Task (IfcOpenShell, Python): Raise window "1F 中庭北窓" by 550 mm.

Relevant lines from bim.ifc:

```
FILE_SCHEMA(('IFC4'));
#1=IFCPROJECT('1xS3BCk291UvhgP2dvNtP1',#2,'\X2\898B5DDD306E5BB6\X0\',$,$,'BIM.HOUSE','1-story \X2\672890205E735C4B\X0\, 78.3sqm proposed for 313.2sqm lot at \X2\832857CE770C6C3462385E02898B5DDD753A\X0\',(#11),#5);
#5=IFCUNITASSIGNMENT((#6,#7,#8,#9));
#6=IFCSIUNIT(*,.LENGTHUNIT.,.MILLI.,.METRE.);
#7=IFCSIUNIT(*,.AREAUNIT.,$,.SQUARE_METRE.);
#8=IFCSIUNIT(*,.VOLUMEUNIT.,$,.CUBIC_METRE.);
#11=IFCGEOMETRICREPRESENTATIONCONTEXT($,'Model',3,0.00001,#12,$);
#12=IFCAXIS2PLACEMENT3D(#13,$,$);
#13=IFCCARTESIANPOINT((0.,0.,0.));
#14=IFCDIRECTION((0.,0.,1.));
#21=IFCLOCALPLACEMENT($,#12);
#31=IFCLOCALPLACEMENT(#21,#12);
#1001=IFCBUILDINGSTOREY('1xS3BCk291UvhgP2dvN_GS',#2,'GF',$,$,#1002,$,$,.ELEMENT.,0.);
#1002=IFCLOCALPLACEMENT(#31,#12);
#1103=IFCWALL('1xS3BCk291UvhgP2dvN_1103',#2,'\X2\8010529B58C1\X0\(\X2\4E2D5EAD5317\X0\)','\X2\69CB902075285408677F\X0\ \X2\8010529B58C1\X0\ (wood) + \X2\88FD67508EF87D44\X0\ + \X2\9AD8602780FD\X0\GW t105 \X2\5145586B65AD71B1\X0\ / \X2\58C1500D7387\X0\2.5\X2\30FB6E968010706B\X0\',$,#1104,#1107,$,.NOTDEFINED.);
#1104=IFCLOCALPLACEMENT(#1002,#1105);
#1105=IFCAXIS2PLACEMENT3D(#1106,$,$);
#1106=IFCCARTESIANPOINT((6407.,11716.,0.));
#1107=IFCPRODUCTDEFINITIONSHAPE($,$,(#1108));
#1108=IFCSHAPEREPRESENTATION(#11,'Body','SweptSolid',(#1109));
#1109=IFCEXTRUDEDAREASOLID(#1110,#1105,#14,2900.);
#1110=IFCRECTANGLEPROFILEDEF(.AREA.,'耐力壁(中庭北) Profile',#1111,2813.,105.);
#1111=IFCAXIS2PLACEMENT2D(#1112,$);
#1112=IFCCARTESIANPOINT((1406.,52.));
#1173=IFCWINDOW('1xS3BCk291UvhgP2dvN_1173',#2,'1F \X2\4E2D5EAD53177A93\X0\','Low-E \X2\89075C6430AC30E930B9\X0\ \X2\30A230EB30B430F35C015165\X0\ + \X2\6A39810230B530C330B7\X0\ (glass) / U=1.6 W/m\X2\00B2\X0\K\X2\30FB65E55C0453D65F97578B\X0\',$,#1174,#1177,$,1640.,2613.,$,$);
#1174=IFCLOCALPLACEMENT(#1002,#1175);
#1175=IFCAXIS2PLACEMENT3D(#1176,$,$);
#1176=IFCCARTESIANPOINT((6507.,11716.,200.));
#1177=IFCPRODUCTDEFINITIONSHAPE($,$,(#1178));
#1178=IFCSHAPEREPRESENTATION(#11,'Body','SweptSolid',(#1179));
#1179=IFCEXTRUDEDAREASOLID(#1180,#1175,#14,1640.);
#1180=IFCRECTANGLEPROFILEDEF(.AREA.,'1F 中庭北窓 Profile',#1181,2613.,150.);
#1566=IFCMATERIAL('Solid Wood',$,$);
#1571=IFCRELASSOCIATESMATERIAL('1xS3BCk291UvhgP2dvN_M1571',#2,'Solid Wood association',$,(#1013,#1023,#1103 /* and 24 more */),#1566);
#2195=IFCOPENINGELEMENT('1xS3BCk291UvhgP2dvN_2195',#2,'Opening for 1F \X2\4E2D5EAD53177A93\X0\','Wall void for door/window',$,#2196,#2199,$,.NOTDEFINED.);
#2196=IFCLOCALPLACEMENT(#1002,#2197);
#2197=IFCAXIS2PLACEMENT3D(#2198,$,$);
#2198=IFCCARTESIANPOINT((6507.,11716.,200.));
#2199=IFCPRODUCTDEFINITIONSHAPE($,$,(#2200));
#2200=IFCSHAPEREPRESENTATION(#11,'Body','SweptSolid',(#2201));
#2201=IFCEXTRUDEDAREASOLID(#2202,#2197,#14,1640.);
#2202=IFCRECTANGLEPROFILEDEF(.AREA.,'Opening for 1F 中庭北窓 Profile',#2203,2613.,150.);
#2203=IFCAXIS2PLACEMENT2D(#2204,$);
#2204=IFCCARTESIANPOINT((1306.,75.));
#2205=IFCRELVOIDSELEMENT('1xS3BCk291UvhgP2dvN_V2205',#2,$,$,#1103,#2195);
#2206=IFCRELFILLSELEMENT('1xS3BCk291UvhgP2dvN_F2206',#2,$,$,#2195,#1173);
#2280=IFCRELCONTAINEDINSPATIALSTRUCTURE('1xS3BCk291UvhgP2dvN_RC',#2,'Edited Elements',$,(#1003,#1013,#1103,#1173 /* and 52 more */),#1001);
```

```python
import numpy as np
import ifcopenshell
import ifcopenshell.api.geometry
import ifcopenshell.util.placement
import ifcopenshell.util.unit

model = ifcopenshell.open("bim.ifc")
unit_scale = ifcopenshell.util.unit.calculate_unit_scale(model)

window = model.by_guid("1xS3BCk291UvhgP2dvN_1173")
opening = window.FillsVoids[0].RelatingOpeningElement
dz = 550.0

shift = np.array([0.0, 0.0, dz])
# The window is not placed relative to its opening, so move both.
for product in (opening, window):
    matrix = ifcopenshell.util.placement.get_local_placement(product.ObjectPlacement)
    matrix[:3, 3] += shift
    ifcopenshell.api.geometry.edit_object_placement(model, product=product, matrix=matrix, is_si=False)

print(f"moved by {dz * unit_scale:+.3f} m")

model.write("bim_updated.ifc")
```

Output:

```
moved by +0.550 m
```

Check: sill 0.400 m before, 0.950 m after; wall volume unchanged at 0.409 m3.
